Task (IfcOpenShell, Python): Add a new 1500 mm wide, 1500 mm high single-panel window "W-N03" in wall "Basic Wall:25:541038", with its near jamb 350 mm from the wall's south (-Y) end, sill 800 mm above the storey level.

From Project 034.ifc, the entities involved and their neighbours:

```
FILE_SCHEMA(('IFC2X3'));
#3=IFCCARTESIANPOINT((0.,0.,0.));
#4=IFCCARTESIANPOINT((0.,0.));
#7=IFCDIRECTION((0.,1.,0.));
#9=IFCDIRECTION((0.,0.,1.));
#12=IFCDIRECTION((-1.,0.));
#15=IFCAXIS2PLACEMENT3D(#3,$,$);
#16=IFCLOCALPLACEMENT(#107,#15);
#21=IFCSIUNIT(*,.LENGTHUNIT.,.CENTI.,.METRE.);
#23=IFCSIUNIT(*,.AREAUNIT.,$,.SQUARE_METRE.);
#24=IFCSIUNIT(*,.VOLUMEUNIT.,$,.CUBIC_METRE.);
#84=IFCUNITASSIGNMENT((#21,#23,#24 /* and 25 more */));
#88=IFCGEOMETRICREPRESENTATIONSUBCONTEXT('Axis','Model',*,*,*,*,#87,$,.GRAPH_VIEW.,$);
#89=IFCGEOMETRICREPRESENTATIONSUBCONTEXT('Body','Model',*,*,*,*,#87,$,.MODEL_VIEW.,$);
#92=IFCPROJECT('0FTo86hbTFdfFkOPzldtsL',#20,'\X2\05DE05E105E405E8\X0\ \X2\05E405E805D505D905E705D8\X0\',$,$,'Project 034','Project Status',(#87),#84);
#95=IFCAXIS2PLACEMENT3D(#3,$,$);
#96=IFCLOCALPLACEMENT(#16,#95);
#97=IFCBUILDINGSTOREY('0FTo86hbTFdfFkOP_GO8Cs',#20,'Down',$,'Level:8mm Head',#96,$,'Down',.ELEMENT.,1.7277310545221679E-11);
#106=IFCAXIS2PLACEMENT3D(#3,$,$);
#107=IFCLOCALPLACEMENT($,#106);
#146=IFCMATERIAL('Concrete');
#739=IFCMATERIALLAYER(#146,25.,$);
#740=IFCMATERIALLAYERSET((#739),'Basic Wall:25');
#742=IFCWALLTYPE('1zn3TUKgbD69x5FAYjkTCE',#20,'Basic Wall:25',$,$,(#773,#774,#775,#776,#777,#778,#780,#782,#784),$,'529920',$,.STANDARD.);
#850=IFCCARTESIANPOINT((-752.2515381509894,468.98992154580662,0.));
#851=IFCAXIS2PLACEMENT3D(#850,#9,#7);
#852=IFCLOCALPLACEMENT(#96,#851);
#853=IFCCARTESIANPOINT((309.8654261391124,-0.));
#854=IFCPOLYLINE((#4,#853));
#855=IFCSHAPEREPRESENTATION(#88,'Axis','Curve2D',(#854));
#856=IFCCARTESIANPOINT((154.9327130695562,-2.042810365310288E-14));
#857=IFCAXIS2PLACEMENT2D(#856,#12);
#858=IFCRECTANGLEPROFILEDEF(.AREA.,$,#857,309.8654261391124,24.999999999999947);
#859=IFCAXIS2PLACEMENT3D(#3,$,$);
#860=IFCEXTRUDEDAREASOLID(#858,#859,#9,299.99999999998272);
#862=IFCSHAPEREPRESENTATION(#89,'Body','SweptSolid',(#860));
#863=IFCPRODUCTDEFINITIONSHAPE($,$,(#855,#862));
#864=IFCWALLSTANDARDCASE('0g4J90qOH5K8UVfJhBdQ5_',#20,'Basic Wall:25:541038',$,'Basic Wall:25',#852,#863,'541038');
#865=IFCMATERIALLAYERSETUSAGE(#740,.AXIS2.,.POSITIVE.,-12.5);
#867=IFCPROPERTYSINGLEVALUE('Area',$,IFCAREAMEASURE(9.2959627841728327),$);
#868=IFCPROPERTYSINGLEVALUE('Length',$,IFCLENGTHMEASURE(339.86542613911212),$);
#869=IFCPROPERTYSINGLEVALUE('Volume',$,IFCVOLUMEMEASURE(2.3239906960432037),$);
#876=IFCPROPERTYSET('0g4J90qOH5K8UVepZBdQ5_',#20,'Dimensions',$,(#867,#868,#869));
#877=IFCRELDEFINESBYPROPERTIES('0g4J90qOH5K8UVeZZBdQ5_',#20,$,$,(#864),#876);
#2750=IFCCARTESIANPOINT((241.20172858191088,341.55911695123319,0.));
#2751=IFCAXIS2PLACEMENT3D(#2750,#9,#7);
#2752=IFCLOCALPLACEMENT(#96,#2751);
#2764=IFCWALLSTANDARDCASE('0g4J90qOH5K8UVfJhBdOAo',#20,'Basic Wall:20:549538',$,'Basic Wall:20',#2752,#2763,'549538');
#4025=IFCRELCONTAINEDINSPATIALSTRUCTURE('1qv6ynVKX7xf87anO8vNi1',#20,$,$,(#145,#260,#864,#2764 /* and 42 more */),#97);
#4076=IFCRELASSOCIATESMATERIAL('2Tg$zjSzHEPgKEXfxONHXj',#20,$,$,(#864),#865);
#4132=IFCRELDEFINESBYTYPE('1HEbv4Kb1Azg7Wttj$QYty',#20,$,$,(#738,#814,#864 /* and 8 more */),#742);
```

```python
import numpy as np
import ifcopenshell
import ifcopenshell.api.feature
import ifcopenshell.api.geometry
import ifcopenshell.api.pset
import ifcopenshell.api.root
import ifcopenshell.api.spatial
import ifcopenshell.api.type
import ifcopenshell.geom
import ifcopenshell.util.element
import ifcopenshell.util.placement
import ifcopenshell.util.representation
import ifcopenshell.util.shape
import ifcopenshell.util.unit

model = ifcopenshell.open("Project 034.ifc")
unit_scale = ifcopenshell.util.unit.calculate_unit_scale(model)
area_scale = ifcopenshell.util.unit.calculate_unit_scale(model, "AREAUNIT")
volume_scale = ifcopenshell.util.unit.calculate_unit_scale(model, "VOLUMEUNIT")
settings = ifcopenshell.geom.settings()


def volume(element):
    """Net volume in cubic metres, openings subtracted."""
    shape = ifcopenshell.geom.create_shape(settings, element)
    return ifcopenshell.util.shape.get_volume(shape.geometry)


wall = model.by_guid("0g4J90qOH5K8UVfJhBdQ5_")
storey = ifcopenshell.util.element.get_container(wall, ifc_class="IfcBuildingStorey")
context = ifcopenshell.util.representation.get_context(model, "Model", "Body", "MODEL_VIEW")
before = volume(wall)

width, height, from_end, sill = 1.5, 1.5, 0.35, 0.8  # metres

# The wall runs along its own X axis, and the end named is its -X end.
wall_shape = ifcopenshell.geom.create_shape(settings, wall)
x, y, z = ifcopenshell.util.shape.get_vertices(wall_shape.geometry).T
start = x.min() + from_end
face, thickness = float(y.min()), float(y.max() - y.min())
wall_matrix = ifcopenshell.util.placement.get_local_placement(wall.ObjectPlacement)
level = ifcopenshell.util.placement.get_local_placement(storey.ObjectPlacement)[2, 3]


def in_wall(x, y):
    """Placement at x, y metres in the wall's axes, at sill height."""
    matrix = wall_matrix.copy()
    matrix[:, 3] = wall_matrix @ np.array([x / unit_scale, y / unit_scale, 0.0, 1.0])
    matrix[2, 3] = level + sill / unit_scale
    return matrix


# Opening: a box that overshoots both wall faces by 50 mm.
opening = ifcopenshell.api.root.create_entity(model, ifc_class="IfcOpeningElement")
box = ifcopenshell.api.geometry.add_wall_representation(
    model, context=context, length=width, height=height, thickness=thickness + 0.1
)
ifcopenshell.api.geometry.assign_representation(model, product=opening, representation=box)
ifcopenshell.api.geometry.edit_object_placement(model, product=opening, matrix=in_wall(start, face - 0.05), is_si=False)
ifcopenshell.api.feature.add_feature(model, feature=opening, element=wall)

window = ifcopenshell.api.root.create_entity(model, ifc_class="IfcWindow", name="W-N03")
window.OverallWidth, window.OverallHeight = width / unit_scale, height / unit_scale
body = ifcopenshell.api.geometry.add_window_representation(
    model,
    context=context,
    overall_width=window.OverallWidth,
    overall_height=window.OverallHeight,
    partition_type="SINGLE_PANEL",
)
ifcopenshell.api.geometry.assign_representation(model, product=window, representation=body)
ifcopenshell.api.spatial.assign_container(model, products=[window], relating_structure=storey)
fills = ifcopenshell.api.feature.add_filling(model, opening=opening, element=window)
fills.OwnerHistory = window.OwnerHistory  # required in IFC2X3

# IFC2X3 keeps the operation on the window style.
style = ifcopenshell.api.root.create_entity(model, ifc_class="IfcWindowStyle", name="W-N03")
style.OperationType, style.ConstructionType = "SINGLE_PANEL", "NOTDEFINED"
style.ParameterTakesPrecedence = style.Sizeable = False
ifcopenshell.api.type.assign_type(model, related_objects=[window], relating_type=style)

# Centre the window in the wall's thickness.
ifcopenshell.api.geometry.edit_object_placement(model, product=window, matrix=in_wall(start, face), is_si=False)
window_shape = ifcopenshell.geom.create_shape(settings, window)
depth = ifcopenshell.util.shape.get_vertices(window_shape.geometry)[:, 1]
offset = face + thickness / 2 - (depth.min() + depth.max()) / 2
ifcopenshell.api.geometry.edit_object_placement(model, product=window, matrix=in_wall(start, offset), is_si=False)

after = volume(wall)

# Update the wall's stored quantities.
pset = model.by_id(ifcopenshell.util.element.get_pset(wall, "Dimensions", should_inherit=False)["id"])
ifcopenshell.api.pset.edit_pset(model, pset=pset, properties={
    "Area": model.create_entity("IfcAreaMeasure", after / thickness / area_scale),
    "Volume": model.create_entity("IfcVolumeMeasure", after / volume_scale),
})

print(f"wall volume {before:.3f} -> {after:.3f} m3")

model.write("Project 034_v2.ifc")
```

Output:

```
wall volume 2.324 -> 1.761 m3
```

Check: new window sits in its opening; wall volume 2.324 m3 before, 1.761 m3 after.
